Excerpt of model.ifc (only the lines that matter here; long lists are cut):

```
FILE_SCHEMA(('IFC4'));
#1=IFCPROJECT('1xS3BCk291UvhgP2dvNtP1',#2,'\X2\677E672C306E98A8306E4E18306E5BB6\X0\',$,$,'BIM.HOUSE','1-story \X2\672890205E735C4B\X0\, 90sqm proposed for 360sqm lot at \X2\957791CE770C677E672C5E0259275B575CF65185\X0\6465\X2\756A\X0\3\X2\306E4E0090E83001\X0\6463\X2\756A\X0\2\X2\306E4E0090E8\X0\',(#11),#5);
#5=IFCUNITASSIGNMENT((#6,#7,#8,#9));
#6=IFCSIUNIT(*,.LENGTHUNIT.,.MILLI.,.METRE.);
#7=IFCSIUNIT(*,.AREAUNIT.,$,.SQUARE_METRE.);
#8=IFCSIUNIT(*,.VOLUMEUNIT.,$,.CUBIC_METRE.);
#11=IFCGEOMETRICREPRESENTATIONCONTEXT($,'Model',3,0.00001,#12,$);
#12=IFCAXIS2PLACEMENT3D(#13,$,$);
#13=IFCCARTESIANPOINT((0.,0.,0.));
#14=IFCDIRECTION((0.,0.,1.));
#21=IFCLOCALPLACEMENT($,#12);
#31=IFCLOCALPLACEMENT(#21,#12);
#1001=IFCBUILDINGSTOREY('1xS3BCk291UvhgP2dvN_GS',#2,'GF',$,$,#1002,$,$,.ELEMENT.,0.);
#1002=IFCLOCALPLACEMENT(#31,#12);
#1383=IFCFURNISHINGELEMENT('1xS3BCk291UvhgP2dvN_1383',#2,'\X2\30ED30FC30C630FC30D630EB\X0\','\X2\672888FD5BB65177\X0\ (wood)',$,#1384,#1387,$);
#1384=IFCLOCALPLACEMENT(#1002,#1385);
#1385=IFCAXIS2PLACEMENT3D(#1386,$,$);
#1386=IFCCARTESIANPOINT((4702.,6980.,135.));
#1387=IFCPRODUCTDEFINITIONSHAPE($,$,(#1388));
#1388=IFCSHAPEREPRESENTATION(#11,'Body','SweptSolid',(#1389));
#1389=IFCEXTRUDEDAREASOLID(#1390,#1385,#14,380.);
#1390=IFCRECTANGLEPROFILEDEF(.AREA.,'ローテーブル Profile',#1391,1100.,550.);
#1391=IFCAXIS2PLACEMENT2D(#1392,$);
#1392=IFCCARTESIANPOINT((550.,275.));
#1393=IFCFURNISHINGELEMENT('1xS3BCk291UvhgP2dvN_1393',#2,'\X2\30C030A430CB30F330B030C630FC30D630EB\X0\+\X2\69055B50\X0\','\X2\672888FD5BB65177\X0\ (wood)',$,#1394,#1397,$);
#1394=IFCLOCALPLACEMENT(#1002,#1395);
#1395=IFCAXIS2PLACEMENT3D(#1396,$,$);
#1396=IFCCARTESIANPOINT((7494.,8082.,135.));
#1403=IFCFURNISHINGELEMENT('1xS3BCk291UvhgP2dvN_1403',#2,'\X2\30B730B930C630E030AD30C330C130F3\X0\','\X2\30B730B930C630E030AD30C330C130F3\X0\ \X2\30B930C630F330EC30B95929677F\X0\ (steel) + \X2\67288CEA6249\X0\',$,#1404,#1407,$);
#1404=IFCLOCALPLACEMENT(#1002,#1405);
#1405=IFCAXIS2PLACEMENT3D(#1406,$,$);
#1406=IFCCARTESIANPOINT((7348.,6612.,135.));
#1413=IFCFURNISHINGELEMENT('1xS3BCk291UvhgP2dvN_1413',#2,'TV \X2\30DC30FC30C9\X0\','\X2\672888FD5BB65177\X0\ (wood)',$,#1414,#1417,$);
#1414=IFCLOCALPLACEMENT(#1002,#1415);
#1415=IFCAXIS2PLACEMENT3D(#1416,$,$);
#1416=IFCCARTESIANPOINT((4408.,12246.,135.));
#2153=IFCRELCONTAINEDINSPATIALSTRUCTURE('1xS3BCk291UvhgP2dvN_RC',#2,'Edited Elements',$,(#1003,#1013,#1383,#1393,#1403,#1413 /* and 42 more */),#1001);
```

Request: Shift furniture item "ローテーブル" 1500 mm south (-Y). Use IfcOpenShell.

```python
import ifcopenshell
import ifcopenshell.api.geometry
import ifcopenshell.util.placement
import ifcopenshell.util.unit

model = ifcopenshell.open("model.ifc")
unit_scale = ifcopenshell.util.unit.calculate_unit_scale(model)

item = model.by_guid("1xS3BCk291UvhgP2dvN_1383")
matrix = ifcopenshell.util.placement.get_local_placement(item.ObjectPlacement)
matrix[1, 3] -= 1.5 / unit_scale
ifcopenshell.api.geometry.edit_object_placement(model, product=item, matrix=matrix, is_si=False)

print(ifcopenshell.util.placement.get_local_placement(item.ObjectPlacement).round(3) + 0.0)

model.write("model_updated.ifc")
```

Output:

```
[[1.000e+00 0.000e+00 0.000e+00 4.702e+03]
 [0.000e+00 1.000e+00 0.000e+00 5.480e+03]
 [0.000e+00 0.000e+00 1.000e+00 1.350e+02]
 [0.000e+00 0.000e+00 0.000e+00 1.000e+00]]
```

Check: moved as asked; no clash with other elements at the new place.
